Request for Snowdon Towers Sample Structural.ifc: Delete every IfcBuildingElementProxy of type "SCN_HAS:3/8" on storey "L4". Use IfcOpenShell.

First a look at what the model holds.

```python
import ifcopenshell
import ifcopenshell.util.element

model = ifcopenshell.open("Snowdon Towers Sample Structural.ifc")
print(model.schema)
storey = next(s for s in model.by_type("IfcBuildingStorey") if s.Name == "L4")
proxies = [e for e in ifcopenshell.util.element.get_decomposition(storey) if e.is_a("IfcBuildingElementProxy")]
seen = {}
for e in proxies:
    element_type = ifcopenshell.util.element.get_type(e)
    name = element_type.Name if element_type not in (None, e) else None
    seen[name] = seen.get(name, 0) + 1
for name, count in sorted(seen.items(), key=str):
    print(count, "x", name)
```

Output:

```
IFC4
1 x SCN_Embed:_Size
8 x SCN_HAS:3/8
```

```python
import ifcopenshell
import ifcopenshell.api.root
import ifcopenshell.util.element

model = ifcopenshell.open("Snowdon Towers Sample Structural.ifc")

storey = next(s for s in model.by_type("IfcBuildingStorey") if s.Name == "L4")
proxies = [e for e in ifcopenshell.util.element.get_decomposition(storey) if e.is_a("IfcBuildingElementProxy")]
targets = [e for e in proxies if (t := ifcopenshell.util.element.get_type(e)) not in (None, e) and t.Name == "SCN_HAS:3/8"]

for e in targets:
    ifcopenshell.api.root.remove_product(model, product=e)
print(len(targets), "removed")

model.write("Snowdon Towers Sample Structural_edited.ifc")
```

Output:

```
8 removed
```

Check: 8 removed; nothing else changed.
